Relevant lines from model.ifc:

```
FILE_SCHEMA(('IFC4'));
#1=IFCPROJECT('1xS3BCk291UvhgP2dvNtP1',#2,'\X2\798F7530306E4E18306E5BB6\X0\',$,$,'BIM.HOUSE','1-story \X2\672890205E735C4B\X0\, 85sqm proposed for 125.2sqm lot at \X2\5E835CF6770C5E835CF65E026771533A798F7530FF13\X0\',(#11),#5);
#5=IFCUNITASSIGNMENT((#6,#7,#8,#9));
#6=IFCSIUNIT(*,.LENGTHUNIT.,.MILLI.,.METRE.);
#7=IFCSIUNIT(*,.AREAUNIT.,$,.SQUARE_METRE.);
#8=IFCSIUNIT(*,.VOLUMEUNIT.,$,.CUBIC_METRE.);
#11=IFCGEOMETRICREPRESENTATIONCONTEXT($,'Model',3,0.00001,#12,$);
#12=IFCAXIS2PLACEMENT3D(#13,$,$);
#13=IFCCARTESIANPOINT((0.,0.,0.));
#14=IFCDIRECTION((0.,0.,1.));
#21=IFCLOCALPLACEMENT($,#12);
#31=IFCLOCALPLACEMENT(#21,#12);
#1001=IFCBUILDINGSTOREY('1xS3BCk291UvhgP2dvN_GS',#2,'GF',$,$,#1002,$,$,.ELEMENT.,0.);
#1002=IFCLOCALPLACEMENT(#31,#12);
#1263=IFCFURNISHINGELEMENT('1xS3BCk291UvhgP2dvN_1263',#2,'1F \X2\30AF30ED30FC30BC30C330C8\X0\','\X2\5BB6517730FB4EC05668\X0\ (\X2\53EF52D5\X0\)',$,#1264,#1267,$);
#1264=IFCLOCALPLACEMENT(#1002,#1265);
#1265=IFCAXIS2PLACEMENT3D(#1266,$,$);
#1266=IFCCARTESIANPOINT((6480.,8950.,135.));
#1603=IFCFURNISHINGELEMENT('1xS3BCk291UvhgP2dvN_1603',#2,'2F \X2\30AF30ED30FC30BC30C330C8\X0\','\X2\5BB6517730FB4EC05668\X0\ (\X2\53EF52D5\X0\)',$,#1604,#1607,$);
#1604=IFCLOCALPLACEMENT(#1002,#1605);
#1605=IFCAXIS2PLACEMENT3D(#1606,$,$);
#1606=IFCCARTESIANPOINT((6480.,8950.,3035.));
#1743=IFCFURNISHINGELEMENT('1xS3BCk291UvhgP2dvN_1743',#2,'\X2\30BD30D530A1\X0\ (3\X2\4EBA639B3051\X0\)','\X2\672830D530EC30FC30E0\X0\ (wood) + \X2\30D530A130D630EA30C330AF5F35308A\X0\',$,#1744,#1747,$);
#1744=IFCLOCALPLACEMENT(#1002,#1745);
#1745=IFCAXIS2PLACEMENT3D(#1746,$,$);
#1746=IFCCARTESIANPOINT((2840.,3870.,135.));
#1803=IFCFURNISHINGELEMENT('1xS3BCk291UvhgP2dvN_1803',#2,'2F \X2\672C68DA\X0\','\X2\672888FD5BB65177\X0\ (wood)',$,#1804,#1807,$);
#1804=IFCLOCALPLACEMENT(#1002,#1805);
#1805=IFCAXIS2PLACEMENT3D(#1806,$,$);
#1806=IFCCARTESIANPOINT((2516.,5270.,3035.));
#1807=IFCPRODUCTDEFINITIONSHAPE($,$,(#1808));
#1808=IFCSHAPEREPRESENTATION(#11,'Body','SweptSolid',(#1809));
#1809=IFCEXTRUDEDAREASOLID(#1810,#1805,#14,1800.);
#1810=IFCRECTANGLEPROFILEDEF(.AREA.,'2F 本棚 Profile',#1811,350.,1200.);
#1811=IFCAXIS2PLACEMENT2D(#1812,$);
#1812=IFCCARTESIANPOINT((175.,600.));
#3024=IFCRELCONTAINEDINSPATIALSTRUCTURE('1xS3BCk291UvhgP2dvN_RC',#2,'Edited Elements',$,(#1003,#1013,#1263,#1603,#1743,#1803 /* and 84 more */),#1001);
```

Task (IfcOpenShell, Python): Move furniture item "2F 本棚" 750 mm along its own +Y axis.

```python
import ifcopenshell
import ifcopenshell.api.geometry
import ifcopenshell.util.placement
import ifcopenshell.util.unit

model = ifcopenshell.open("model.ifc")
unit_scale = ifcopenshell.util.unit.calculate_unit_scale(model)

item = model.by_guid("1xS3BCk291UvhgP2dvN_1803")
matrix = ifcopenshell.util.placement.get_local_placement(item.ObjectPlacement)
matrix[:3, 3] += matrix[:3, 1] * 0.75 / unit_scale
ifcopenshell.api.geometry.edit_object_placement(model, product=item, matrix=matrix, is_si=False)

print(ifcopenshell.util.placement.get_local_placement(item.ObjectPlacement).round(3) + 0.0)

model.write("model_rev.ifc")
```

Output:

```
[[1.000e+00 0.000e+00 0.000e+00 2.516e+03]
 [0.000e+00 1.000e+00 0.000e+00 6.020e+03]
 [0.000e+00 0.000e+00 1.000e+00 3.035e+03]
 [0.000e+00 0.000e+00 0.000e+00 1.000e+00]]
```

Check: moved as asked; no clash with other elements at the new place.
